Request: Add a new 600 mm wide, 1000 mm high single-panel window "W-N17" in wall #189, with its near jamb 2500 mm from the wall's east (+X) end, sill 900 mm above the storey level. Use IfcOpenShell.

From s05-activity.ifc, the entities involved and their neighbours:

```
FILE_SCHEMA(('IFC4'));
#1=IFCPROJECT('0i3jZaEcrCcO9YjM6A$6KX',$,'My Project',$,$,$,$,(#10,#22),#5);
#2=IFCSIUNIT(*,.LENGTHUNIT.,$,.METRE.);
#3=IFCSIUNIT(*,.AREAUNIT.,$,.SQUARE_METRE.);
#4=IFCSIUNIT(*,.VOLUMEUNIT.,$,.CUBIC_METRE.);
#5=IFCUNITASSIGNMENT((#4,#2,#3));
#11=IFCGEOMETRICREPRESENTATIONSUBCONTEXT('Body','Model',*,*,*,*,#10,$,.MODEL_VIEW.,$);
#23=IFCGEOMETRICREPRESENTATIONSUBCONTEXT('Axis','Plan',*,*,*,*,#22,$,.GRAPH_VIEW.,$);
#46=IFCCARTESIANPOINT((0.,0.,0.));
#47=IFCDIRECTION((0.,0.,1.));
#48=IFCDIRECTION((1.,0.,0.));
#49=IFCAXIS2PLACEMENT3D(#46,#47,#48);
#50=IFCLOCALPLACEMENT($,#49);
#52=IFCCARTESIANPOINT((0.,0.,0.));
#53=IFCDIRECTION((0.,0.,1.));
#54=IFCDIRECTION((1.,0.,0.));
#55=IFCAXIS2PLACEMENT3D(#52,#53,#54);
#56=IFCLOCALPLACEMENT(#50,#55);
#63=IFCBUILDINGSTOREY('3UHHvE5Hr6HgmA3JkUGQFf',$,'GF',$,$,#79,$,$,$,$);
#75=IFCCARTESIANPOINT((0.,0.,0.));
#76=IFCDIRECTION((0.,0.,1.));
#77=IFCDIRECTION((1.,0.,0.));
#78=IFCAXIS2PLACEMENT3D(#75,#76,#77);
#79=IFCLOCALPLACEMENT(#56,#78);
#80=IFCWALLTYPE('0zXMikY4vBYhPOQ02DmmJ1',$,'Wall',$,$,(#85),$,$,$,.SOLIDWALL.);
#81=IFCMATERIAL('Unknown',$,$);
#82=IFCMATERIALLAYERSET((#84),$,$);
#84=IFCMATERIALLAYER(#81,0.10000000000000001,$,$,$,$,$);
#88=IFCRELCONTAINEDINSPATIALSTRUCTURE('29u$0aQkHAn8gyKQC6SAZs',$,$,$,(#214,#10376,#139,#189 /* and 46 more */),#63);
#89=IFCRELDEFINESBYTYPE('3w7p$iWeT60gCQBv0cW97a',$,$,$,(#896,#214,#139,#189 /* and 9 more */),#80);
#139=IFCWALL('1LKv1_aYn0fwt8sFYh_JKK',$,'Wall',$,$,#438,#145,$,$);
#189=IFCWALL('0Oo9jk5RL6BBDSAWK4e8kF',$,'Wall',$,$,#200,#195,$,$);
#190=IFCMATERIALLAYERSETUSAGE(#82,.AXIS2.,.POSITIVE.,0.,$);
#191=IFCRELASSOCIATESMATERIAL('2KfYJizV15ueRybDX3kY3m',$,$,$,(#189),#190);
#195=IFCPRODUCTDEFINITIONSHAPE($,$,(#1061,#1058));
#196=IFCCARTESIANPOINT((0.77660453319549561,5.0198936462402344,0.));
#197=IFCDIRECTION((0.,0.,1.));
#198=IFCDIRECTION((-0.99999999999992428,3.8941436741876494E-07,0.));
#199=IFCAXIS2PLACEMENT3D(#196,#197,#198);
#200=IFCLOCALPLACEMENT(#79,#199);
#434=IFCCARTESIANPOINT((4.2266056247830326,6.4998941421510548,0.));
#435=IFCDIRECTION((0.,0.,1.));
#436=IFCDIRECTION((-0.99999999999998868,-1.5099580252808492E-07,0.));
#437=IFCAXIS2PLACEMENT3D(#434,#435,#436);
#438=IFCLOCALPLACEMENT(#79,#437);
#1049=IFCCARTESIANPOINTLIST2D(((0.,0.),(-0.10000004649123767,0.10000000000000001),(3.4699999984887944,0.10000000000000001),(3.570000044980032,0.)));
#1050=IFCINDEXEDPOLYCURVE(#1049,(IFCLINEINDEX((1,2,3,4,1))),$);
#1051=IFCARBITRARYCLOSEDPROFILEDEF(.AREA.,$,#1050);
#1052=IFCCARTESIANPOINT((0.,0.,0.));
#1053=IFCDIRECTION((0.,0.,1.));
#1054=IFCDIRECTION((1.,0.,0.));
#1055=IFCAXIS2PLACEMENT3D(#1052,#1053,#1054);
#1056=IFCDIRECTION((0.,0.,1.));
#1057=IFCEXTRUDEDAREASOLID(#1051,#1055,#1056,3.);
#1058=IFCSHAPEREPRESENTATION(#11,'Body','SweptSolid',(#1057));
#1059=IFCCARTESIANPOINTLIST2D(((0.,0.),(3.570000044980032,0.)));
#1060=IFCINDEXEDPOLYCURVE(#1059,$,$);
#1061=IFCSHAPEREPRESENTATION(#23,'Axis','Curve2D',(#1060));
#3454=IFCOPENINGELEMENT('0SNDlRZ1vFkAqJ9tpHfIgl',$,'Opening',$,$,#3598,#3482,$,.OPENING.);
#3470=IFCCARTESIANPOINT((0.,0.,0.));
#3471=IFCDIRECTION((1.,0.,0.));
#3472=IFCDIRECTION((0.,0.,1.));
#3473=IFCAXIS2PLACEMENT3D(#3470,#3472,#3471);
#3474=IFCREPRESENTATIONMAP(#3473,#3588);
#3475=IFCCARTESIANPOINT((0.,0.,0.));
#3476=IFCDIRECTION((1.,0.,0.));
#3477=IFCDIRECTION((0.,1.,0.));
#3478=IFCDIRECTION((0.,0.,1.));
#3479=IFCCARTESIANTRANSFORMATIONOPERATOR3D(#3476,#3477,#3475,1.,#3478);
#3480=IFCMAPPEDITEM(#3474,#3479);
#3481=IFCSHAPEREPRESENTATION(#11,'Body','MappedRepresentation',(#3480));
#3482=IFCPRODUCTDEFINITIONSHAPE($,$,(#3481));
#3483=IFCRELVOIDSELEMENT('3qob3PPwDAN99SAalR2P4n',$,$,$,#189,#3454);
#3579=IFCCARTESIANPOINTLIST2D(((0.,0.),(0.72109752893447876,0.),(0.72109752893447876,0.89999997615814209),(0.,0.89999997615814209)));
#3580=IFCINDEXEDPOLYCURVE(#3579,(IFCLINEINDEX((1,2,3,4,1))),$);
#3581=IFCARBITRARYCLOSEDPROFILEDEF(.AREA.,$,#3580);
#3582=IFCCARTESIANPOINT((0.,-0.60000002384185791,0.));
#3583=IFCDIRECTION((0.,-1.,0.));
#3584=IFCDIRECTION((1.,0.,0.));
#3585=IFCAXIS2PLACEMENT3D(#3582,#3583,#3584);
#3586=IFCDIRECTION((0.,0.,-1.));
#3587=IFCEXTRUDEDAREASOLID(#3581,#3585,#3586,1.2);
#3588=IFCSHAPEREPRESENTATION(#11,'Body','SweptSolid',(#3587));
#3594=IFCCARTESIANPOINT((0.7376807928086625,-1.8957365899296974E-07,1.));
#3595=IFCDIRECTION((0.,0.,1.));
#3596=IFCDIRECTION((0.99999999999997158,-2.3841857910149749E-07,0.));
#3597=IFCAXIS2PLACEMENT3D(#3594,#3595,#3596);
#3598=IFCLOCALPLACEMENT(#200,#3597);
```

```python
import numpy as np
import ifcopenshell
import ifcopenshell.api.feature
import ifcopenshell.api.geometry
import ifcopenshell.api.root
import ifcopenshell.api.spatial
import ifcopenshell.geom
import ifcopenshell.util.element
import ifcopenshell.util.placement
import ifcopenshell.util.representation
import ifcopenshell.util.shape
import ifcopenshell.util.unit

model = ifcopenshell.open("s05-activity.ifc")
unit_scale = ifcopenshell.util.unit.calculate_unit_scale(model)
settings = ifcopenshell.geom.settings()


def volume(element):
    """Net volume in cubic metres, openings subtracted."""
    shape = ifcopenshell.geom.create_shape(settings, element)
    return ifcopenshell.util.shape.get_volume(shape.geometry)


wall = model.by_guid("0Oo9jk5RL6BBDSAWK4e8kF")
storey = ifcopenshell.util.element.get_container(wall, ifc_class="IfcBuildingStorey")
context = ifcopenshell.util.representation.get_context(model, "Model", "Body", "MODEL_VIEW")
before = volume(wall)

width, height, from_end, sill = 0.6, 1, 2.5, 0.9  # metres

# The wall runs along its own X axis, and the end named is its -X end.
wall_shape = ifcopenshell.geom.create_shape(settings, wall)
x, y, z = ifcopenshell.util.shape.get_vertices(wall_shape.geometry).T
start = x.min() + from_end
face, thickness = float(y.min()), float(y.max() - y.min())
wall_matrix = ifcopenshell.util.placement.get_local_placement(wall.ObjectPlacement)
level = ifcopenshell.util.placement.get_local_placement(storey.ObjectPlacement)[2, 3]


def in_wall(x, y):
    """Placement at x, y metres in the wall's axes, at sill height."""
    matrix = wall_matrix.copy()
    matrix[:, 3] = wall_matrix @ np.array([x / unit_scale, y / unit_scale, 0.0, 1.0])
    matrix[2, 3] = level + sill / unit_scale
    return matrix


# Opening: a box that overshoots both wall faces by 50 mm.
opening = ifcopenshell.api.root.create_entity(model, ifc_class="IfcOpeningElement", predefined_type="OPENING")
box = ifcopenshell.api.geometry.add_wall_representation(
    model, context=context, length=width, height=height, thickness=thickness + 0.1
)
ifcopenshell.api.geometry.assign_representation(model, product=opening, representation=box)
ifcopenshell.api.geometry.edit_object_placement(model, product=opening, matrix=in_wall(start, face - 0.05), is_si=False)
ifcopenshell.api.feature.add_feature(model, feature=opening, element=wall)

window = ifcopenshell.api.root.create_entity(model, ifc_class="IfcWindow", name="W-N17", predefined_type="WINDOW")
window.OverallWidth, window.OverallHeight = width / unit_scale, height / unit_scale
window.PartitioningType = "SINGLE_PANEL"
body = ifcopenshell.api.geometry.add_window_representation(
    model,
    context=context,
    overall_width=window.OverallWidth,
    overall_height=window.OverallHeight,
    partition_type="SINGLE_PANEL",
)
ifcopenshell.api.geometry.assign_representation(model, product=window, representation=body)
ifcopenshell.api.spatial.assign_container(model, products=[window], relating_structure=storey)
ifcopenshell.api.feature.add_filling(model, opening=opening, element=window)

# Centre the window in the wall's thickness.
ifcopenshell.api.geometry.edit_object_placement(model, product=window, matrix=in_wall(start, face), is_si=False)
window_shape = ifcopenshell.geom.create_shape(settings, window)
depth = ifcopenshell.util.shape.get_vertices(window_shape.geometry)[:, 1]
offset = face + thickness / 2 - (depth.min() + depth.max()) / 2
ifcopenshell.api.geometry.edit_object_placement(model, product=window, matrix=in_wall(start, offset), is_si=False)

after = volume(wall)

print(f"wall volume {before:.3f} -> {after:.3f} m3")

model.write("s05-activity_edited.ifc")
```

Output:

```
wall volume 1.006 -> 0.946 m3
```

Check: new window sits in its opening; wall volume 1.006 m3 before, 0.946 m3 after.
